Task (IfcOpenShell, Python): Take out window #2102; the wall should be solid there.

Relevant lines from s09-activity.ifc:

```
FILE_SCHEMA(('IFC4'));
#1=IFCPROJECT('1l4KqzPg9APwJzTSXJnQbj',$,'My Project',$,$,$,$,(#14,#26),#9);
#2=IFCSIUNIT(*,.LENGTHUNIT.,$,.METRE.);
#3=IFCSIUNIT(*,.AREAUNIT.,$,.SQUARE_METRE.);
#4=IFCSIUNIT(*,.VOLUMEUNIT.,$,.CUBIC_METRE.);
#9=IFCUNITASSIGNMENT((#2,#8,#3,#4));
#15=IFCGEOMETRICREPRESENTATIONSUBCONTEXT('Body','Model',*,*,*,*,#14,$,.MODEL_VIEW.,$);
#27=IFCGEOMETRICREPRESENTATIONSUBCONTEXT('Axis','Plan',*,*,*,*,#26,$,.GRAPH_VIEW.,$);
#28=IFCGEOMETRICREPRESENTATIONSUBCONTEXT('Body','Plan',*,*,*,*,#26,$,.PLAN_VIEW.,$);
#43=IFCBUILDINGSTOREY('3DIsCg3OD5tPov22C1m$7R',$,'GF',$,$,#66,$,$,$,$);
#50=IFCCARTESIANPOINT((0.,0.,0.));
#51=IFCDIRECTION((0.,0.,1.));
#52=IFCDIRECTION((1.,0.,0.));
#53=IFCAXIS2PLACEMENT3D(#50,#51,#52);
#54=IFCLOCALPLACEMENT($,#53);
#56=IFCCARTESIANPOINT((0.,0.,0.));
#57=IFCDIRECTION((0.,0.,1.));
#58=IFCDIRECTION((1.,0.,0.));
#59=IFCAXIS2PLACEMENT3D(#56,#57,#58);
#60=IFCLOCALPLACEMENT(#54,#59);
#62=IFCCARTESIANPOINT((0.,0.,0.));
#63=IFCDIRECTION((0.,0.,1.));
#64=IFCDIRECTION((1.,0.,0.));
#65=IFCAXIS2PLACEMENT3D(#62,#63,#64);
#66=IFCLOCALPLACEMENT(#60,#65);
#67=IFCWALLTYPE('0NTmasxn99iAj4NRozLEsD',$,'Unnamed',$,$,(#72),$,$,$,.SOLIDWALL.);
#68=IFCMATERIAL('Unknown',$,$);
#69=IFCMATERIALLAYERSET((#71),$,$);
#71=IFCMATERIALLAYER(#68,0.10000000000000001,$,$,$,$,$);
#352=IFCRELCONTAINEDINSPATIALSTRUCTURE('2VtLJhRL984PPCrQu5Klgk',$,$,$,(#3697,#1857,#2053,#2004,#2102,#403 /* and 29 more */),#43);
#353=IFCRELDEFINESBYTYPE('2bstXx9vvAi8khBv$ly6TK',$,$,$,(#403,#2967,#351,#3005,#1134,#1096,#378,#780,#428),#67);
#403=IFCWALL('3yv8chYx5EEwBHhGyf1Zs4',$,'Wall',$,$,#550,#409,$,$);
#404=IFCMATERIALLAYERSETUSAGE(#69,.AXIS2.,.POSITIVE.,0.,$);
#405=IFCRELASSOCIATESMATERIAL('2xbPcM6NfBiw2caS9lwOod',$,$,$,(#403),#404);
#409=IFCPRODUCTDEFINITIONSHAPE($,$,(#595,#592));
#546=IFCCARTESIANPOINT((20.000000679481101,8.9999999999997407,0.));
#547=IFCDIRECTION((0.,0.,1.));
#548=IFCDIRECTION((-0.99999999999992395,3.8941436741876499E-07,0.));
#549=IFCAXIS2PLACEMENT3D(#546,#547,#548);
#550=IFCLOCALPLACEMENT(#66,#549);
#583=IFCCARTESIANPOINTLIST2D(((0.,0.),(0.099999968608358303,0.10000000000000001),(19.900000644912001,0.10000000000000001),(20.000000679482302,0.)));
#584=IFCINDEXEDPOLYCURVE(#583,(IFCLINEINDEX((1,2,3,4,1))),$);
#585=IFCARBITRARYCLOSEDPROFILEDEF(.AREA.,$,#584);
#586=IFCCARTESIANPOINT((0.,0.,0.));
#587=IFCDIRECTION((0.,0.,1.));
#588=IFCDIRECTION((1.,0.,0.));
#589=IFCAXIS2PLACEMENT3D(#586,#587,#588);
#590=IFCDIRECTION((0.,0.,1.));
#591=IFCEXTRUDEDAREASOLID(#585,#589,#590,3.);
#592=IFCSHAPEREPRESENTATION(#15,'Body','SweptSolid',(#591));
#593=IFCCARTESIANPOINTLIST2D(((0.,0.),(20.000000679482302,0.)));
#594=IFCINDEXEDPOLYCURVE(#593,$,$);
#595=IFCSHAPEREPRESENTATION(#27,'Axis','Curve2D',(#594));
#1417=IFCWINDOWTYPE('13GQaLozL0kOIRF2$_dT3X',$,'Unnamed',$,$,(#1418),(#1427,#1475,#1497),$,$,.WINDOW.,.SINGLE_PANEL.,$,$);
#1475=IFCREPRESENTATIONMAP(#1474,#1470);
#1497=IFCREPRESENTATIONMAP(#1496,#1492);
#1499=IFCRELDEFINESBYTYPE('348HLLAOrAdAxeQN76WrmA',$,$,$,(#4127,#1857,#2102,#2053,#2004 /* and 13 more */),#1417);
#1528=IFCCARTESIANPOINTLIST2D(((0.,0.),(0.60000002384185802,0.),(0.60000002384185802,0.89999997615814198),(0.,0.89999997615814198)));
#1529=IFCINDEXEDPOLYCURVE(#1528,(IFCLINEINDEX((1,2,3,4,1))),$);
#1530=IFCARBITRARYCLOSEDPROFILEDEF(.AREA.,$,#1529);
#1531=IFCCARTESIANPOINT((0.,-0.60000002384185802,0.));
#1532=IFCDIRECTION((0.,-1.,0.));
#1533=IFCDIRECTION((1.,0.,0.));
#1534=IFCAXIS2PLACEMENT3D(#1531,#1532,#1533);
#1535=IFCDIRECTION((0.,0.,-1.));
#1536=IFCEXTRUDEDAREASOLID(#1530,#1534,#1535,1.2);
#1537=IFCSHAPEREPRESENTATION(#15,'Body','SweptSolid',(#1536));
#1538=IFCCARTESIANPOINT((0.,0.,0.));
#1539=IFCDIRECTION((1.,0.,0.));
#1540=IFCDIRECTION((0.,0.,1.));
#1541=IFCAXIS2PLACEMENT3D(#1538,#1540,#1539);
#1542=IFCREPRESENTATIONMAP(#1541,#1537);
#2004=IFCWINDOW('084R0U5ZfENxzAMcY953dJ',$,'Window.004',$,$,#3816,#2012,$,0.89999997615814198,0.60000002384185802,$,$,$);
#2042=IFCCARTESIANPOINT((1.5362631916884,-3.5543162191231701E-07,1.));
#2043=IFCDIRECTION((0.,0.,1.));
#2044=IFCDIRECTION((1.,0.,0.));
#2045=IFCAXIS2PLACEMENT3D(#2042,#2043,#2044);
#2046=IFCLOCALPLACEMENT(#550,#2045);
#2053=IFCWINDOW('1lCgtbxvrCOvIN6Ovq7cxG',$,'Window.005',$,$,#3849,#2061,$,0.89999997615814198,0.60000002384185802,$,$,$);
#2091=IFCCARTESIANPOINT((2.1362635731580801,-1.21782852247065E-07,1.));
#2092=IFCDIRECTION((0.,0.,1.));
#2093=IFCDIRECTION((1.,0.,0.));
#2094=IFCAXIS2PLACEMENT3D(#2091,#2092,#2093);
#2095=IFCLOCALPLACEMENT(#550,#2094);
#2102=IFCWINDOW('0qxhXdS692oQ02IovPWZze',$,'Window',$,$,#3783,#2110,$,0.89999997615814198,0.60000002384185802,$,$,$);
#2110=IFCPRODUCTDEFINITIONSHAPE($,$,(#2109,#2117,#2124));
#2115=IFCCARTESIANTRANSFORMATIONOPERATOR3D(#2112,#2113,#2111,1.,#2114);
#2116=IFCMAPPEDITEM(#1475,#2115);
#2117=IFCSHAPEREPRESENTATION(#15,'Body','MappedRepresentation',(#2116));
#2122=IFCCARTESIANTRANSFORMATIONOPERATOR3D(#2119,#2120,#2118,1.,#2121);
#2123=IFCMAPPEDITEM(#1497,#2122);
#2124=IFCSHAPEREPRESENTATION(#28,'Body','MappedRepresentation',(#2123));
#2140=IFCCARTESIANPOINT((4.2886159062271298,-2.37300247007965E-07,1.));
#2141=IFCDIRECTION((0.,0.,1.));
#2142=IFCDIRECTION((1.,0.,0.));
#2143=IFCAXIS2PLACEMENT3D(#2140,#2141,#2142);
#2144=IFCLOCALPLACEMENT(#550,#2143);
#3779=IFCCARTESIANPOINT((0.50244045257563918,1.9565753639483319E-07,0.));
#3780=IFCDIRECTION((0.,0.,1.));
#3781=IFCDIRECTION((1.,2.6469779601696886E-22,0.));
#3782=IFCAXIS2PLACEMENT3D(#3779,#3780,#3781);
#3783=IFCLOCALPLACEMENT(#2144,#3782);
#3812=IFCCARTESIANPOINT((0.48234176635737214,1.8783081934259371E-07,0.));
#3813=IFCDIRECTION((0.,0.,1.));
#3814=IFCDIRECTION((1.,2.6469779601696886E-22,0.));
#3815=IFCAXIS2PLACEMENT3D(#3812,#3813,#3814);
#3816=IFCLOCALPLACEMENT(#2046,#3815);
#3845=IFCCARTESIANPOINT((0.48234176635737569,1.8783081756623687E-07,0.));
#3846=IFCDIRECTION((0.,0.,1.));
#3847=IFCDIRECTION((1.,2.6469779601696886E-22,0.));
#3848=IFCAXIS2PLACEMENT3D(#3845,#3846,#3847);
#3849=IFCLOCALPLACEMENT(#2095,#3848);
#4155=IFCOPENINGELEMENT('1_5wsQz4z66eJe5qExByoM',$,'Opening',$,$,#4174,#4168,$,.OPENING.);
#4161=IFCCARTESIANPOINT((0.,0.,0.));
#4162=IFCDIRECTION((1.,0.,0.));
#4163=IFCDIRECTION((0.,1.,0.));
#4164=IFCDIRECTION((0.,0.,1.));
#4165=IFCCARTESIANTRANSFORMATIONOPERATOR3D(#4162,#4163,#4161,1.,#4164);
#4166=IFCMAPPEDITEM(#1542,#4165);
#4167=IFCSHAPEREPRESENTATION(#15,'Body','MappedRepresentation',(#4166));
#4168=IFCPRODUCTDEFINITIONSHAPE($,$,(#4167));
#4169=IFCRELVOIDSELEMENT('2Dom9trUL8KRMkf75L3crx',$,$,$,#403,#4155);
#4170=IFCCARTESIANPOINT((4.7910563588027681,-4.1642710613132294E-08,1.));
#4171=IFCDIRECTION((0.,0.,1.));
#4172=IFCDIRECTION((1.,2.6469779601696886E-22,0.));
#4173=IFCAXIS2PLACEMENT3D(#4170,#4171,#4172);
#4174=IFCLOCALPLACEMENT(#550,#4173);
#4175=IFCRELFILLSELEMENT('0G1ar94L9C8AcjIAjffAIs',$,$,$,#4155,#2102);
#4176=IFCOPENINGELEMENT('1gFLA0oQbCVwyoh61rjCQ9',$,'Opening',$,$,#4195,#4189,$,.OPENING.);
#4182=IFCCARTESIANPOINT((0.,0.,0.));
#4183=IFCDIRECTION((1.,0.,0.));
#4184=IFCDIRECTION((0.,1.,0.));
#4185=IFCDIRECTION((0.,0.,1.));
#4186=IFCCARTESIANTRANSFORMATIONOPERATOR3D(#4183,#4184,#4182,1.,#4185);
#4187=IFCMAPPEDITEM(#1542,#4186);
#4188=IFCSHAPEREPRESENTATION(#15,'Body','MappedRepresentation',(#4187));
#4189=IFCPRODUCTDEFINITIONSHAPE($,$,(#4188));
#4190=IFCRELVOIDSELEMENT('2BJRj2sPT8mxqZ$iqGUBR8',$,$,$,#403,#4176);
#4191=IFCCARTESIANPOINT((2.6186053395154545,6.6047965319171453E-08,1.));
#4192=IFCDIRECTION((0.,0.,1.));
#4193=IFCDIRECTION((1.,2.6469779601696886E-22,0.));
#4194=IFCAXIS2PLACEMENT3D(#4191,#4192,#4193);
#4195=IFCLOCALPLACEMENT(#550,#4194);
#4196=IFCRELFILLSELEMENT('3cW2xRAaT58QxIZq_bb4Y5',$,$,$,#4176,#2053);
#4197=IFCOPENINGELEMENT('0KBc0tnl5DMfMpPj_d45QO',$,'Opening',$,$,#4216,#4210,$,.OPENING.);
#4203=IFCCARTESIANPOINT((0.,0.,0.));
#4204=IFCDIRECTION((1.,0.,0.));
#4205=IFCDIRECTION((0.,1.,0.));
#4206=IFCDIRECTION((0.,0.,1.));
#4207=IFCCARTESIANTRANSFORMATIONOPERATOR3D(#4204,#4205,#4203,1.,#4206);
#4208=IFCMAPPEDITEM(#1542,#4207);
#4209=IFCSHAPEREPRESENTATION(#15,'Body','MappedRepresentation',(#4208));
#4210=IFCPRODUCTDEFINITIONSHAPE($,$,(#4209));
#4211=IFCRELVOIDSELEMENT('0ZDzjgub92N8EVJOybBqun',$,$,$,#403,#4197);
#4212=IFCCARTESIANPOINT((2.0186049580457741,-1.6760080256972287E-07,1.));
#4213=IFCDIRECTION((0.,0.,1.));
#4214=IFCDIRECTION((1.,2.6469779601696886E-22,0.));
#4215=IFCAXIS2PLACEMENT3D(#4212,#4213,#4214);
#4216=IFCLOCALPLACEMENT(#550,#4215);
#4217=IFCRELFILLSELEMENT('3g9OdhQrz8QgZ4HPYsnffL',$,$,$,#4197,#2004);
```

```python
import ifcopenshell
import ifcopenshell.api.feature
import ifcopenshell.api.root
import ifcopenshell.geom
import ifcopenshell.util.shape

model = ifcopenshell.open("s09-activity.ifc")
settings = ifcopenshell.geom.settings()


def volume(element):
    """Net volume in cubic metres, openings subtracted."""
    shape = ifcopenshell.geom.create_shape(settings, element)
    return ifcopenshell.util.shape.get_volume(shape.geometry)


window = model.by_guid("0qxhXdS692oQ02IovPWZze")
opening = window.FillsVoids[0].RelatingOpeningElement
wall = opening.VoidsElements[0].RelatingBuildingElement
before = volume(wall)

ifcopenshell.api.root.remove_product(model, product=window)
ifcopenshell.api.feature.remove_feature(model, feature=opening)

after = volume(wall)

print(f"wall volume {before:.3f} -> {after:.3f} m3")

model.write("s09-activity_v2.ifc")
```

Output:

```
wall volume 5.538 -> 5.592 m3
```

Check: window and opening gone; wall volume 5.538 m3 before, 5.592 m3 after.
